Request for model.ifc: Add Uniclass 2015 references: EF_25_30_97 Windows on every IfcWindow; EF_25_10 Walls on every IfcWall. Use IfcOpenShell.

First a look at what the model holds.

```python
import ifcopenshell

model = ifcopenshell.open("model.ifc")
print(model.schema)
print("classifications:", [c.Name for c in model.by_type("IfcClassification")])
for ifc_class in ("IfcDoor", "IfcRoof", "IfcStair", "IfcWall", "IfcWindow"):
    print(ifc_class, len(model.by_type(ifc_class)))
```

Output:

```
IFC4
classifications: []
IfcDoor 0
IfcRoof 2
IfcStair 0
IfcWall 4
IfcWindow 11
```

```python
import ifcopenshell
import ifcopenshell.api.classification

model = ifcopenshell.open("model.ifc")

system = ifcopenshell.api.classification.add_classification(model, classification="Uniclass 2015")

codes = {
    "IfcWindow": ("EF_25_30_97", "Windows"),
    "IfcWall": ("EF_25_10", "Walls"),
}
for ifc_class, (code, name) in codes.items():
    products = model.by_type(ifc_class)
    ifcopenshell.api.classification.add_reference(
        model, products=products, classification=system, identification=code, name=name
    )
    print(code, len(products))

model.write("model-out.ifc")
```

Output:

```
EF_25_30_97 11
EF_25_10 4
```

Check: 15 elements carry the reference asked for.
